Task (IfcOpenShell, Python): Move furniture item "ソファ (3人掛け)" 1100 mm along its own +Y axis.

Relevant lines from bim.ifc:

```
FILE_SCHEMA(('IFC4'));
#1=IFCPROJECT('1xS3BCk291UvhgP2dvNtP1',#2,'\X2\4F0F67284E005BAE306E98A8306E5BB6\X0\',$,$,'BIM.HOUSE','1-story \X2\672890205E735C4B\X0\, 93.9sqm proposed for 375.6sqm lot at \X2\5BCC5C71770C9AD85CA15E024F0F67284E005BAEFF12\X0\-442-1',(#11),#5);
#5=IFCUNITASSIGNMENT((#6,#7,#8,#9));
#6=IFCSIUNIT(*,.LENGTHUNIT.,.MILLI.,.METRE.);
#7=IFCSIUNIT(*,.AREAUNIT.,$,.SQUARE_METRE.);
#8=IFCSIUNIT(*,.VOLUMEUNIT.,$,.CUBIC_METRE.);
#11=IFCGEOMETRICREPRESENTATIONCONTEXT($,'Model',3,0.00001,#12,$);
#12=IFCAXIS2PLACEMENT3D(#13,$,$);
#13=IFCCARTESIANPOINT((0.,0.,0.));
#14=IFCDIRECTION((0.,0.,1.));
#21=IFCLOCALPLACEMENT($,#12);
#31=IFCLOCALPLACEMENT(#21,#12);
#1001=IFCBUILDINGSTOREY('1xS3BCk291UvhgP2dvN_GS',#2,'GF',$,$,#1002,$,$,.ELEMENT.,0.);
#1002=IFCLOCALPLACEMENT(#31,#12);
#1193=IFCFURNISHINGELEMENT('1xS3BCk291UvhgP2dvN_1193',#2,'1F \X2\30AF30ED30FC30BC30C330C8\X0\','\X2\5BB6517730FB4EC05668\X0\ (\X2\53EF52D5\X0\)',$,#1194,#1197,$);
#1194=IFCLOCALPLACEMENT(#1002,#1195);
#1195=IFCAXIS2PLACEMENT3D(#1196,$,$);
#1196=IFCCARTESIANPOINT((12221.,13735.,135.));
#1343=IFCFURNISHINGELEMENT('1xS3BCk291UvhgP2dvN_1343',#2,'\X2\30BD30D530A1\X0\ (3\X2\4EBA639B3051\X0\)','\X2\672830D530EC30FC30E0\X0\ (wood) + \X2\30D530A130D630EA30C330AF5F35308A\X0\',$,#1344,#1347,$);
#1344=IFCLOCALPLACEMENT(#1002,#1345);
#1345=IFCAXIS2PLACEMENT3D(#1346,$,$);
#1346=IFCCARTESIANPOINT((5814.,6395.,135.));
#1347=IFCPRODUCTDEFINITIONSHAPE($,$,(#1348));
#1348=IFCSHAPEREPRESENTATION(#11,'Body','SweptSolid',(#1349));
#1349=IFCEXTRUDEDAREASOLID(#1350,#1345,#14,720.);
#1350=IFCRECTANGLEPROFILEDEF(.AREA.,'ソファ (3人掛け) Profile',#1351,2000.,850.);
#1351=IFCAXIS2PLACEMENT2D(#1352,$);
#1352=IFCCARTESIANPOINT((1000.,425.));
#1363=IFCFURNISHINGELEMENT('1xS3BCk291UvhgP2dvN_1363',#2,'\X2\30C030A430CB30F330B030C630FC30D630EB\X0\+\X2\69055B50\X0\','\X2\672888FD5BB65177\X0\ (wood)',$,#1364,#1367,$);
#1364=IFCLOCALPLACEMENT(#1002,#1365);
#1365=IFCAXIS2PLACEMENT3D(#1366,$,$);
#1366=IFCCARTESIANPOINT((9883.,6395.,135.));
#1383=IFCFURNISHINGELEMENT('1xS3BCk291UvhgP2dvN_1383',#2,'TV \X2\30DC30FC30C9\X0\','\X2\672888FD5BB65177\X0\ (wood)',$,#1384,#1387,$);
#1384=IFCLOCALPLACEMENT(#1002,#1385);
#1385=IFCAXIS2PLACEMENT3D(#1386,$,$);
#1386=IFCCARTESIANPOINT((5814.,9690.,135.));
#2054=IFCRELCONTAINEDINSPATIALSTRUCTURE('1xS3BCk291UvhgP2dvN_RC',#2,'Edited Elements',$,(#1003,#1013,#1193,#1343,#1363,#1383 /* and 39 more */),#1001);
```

```python
import ifcopenshell
import ifcopenshell.api.geometry
import ifcopenshell.util.placement
import ifcopenshell.util.unit

model = ifcopenshell.open("bim.ifc")
unit_scale = ifcopenshell.util.unit.calculate_unit_scale(model)

item = model.by_id(1343)
matrix = ifcopenshell.util.placement.get_local_placement(item.ObjectPlacement)
matrix[:3, 3] += matrix[:3, 1] * 1.1 / unit_scale
ifcopenshell.api.geometry.edit_object_placement(model, product=item, matrix=matrix, is_si=False)

print(ifcopenshell.util.placement.get_local_placement(item.ObjectPlacement).round(3) + 0.0)

model.write("bim_edited.ifc")
```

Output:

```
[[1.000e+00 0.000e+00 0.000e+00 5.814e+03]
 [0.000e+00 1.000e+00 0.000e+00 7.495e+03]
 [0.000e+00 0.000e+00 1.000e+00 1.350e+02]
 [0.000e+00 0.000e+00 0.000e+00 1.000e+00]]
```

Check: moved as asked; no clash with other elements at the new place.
